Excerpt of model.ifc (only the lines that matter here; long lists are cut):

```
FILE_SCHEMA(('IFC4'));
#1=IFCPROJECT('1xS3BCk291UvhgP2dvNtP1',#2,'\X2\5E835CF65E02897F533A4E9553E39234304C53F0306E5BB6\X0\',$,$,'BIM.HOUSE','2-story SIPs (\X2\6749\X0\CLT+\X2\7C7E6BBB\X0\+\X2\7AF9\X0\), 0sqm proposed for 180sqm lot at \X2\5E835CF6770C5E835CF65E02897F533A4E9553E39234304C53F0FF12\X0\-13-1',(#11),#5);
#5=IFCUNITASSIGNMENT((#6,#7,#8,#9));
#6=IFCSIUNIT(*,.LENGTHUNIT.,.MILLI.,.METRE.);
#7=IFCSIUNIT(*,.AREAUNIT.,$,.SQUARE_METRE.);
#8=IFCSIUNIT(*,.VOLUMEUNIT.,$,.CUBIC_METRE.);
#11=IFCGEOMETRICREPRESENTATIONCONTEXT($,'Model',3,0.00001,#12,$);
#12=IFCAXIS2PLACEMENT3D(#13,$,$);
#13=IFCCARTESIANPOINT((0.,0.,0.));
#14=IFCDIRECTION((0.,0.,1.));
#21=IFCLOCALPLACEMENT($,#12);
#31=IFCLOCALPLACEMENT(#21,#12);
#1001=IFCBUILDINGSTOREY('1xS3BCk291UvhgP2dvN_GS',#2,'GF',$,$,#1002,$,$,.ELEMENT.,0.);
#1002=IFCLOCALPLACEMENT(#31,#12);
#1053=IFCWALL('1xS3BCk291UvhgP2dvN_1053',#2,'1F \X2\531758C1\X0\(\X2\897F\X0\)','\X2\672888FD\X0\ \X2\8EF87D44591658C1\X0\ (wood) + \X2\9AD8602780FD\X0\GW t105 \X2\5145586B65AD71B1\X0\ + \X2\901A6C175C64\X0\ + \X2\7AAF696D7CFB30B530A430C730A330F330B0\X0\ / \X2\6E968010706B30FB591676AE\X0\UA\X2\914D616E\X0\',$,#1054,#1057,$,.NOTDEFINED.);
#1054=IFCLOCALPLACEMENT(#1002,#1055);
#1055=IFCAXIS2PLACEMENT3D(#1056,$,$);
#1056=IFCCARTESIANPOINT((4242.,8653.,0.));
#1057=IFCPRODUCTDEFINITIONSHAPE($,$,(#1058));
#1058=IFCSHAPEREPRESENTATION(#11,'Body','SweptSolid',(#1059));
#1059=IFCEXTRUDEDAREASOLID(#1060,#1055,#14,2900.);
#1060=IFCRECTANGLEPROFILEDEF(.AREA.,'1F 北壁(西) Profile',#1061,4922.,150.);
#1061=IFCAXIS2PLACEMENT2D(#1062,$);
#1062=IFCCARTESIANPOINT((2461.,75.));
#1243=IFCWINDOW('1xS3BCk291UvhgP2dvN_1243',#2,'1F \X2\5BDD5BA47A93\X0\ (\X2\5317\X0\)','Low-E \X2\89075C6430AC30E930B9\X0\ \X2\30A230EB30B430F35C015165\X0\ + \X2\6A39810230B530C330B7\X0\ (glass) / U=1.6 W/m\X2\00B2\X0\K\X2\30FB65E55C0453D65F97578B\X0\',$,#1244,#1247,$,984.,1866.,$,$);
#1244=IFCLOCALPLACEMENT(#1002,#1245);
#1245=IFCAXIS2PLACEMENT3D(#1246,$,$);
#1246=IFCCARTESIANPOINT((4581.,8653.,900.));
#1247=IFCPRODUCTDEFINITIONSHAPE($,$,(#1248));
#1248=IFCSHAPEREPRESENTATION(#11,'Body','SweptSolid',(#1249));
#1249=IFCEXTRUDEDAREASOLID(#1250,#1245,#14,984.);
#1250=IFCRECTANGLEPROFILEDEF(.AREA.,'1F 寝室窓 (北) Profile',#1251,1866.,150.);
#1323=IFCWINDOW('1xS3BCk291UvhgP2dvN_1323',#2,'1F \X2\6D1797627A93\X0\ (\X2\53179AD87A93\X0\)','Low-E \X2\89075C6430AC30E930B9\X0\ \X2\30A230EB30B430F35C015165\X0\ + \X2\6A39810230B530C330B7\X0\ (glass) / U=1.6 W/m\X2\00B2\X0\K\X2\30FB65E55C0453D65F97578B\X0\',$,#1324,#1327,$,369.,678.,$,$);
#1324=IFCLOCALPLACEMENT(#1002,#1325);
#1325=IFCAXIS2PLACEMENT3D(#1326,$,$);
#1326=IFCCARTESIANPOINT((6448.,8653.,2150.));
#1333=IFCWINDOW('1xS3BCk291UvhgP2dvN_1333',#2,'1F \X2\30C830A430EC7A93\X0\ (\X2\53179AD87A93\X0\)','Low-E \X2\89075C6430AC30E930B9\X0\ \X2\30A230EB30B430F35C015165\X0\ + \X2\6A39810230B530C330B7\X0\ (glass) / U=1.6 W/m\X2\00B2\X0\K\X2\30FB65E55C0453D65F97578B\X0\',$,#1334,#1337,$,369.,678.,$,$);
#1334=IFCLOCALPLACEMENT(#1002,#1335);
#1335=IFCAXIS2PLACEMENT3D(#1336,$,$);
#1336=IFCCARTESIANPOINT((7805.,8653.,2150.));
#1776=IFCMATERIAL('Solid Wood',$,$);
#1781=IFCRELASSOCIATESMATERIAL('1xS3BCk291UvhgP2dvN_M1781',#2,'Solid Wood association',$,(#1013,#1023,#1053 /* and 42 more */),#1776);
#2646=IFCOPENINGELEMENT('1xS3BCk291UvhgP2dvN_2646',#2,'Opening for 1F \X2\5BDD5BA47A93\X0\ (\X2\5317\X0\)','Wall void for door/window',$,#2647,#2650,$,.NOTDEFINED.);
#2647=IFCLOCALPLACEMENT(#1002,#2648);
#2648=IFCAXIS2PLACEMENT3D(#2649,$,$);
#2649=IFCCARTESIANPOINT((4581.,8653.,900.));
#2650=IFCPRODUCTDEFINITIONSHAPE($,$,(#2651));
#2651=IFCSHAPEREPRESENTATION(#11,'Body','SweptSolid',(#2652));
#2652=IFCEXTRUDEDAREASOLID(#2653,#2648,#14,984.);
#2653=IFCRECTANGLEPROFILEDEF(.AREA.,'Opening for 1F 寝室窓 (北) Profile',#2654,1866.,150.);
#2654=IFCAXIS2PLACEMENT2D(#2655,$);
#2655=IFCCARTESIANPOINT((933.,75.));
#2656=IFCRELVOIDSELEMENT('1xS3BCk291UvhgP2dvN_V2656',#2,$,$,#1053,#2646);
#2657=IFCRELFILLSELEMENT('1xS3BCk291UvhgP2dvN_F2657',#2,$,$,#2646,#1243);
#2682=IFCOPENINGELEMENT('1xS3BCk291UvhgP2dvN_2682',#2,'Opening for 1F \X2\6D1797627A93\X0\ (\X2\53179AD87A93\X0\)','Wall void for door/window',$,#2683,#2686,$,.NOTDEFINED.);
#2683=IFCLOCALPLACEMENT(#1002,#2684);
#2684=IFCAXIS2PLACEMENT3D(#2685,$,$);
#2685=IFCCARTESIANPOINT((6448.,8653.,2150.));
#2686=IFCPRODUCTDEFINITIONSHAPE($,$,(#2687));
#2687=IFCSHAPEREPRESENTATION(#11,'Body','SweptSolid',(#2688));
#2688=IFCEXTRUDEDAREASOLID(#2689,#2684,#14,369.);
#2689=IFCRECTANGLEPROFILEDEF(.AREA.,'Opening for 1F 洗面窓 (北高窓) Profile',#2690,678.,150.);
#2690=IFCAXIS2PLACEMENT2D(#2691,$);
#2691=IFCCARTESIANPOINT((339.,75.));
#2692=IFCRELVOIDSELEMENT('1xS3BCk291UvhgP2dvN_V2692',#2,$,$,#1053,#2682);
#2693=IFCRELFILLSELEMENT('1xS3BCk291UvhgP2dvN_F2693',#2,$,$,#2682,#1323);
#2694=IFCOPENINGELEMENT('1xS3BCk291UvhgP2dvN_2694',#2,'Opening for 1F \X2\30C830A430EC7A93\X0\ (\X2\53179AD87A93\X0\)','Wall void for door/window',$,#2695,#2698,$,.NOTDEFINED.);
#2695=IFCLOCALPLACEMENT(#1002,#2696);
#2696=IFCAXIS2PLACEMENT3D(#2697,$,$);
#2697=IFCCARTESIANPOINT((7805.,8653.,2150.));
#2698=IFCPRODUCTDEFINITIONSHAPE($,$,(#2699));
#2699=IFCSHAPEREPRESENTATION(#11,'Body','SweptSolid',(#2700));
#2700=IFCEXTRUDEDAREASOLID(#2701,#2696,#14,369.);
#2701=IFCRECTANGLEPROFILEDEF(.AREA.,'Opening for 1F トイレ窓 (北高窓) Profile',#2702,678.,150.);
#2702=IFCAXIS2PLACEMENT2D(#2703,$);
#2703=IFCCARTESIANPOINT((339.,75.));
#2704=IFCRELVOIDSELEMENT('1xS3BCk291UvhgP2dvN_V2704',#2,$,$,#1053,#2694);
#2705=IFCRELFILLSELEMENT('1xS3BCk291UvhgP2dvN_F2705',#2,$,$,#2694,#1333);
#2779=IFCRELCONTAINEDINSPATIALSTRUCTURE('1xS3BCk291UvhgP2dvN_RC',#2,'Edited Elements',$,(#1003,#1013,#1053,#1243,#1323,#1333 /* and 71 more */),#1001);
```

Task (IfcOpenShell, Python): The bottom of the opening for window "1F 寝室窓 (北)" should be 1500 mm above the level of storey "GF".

```python
import numpy as np
import ifcopenshell
import ifcopenshell.api.geometry
import ifcopenshell.geom
import ifcopenshell.util.element
import ifcopenshell.util.placement
import ifcopenshell.util.shape
import ifcopenshell.util.unit

model = ifcopenshell.open("model.ifc")
unit_scale = ifcopenshell.util.unit.calculate_unit_scale(model)

window = model.by_id(1243)
opening = window.FillsVoids[0].RelatingOpeningElement
storey = ifcopenshell.util.element.get_container(window, ifc_class="IfcBuildingStorey")
level = ifcopenshell.util.placement.get_local_placement(storey.ObjectPlacement)[2, 3]

# The opening's origin need not be at the sill, so measure its lowest point.
shape = ifcopenshell.geom.create_shape(ifcopenshell.geom.settings(), opening)
bottom = ifcopenshell.util.shape.get_shape_bottom_elevation(shape, shape.geometry) / unit_scale
dz = level + 1500.0 - bottom

shift = np.array([0.0, 0.0, dz])
# The window is not placed relative to its opening, so move both.
for product in (opening, window):
    matrix = ifcopenshell.util.placement.get_local_placement(product.ObjectPlacement)
    matrix[:3, 3] += shift
    ifcopenshell.api.geometry.edit_object_placement(model, product=product, matrix=matrix, is_si=False)

print(f"moved by {dz * unit_scale:+.3f} m")

model.write("model_rev.ifc")
```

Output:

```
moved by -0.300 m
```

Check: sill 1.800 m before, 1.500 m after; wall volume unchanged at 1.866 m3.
